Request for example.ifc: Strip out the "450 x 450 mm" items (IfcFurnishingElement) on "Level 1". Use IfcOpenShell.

First a look at what the model holds.

```python
import ifcopenshell
import ifcopenshell.util.element

model = ifcopenshell.open("example.ifc")
print(model.schema)
storey = next(s for s in model.by_type("IfcBuildingStorey") if s.Name == "Level 1")
furniture = [e for e in ifcopenshell.util.element.get_decomposition(storey) if e.is_a("IfcFurnishingElement")]
seen = {}
for e in furniture:
    element_type = ifcopenshell.util.element.get_type(e)
    name = element_type.Name if element_type not in (None, e) else None
    seen[name] = seen.get(name, 0) + 1
for name, count in sorted(seen.items(), key=str):
    print(count, "x", name)
```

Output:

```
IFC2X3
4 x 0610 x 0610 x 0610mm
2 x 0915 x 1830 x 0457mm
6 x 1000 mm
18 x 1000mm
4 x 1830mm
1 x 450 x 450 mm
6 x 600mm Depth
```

```python
import ifcopenshell
import ifcopenshell.api.root
import ifcopenshell.util.element

model = ifcopenshell.open("example.ifc")

storey = next(s for s in model.by_type("IfcBuildingStorey") if s.Name == "Level 1")
furniture = [e for e in ifcopenshell.util.element.get_decomposition(storey) if e.is_a("IfcFurnishingElement")]
targets = [e for e in furniture if (t := ifcopenshell.util.element.get_type(e)) not in (None, e) and t.Name == "450 x 450 mm"]

for e in targets:
    ifcopenshell.api.root.remove_product(model, product=e)
print(len(targets), "removed")

model.write("example-out.ifc")
```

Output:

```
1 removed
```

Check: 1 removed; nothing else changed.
